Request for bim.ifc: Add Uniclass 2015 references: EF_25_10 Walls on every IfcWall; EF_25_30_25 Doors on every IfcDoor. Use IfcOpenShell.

First a look at what the model holds.

```python
import ifcopenshell

model = ifcopenshell.open("bim.ifc")
print(model.schema)
print("classifications:", [c.Name for c in model.by_type("IfcClassification")])
for ifc_class in ("IfcDoor", "IfcRoof", "IfcStair", "IfcWall", "IfcWindow"):
    print(ifc_class, len(model.by_type(ifc_class)))
```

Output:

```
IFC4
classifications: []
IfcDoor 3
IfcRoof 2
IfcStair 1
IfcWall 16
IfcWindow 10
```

```python
import ifcopenshell
import ifcopenshell.api.classification

model = ifcopenshell.open("bim.ifc")

system = ifcopenshell.api.classification.add_classification(model, classification="Uniclass 2015")

codes = {
    "IfcWall": ("EF_25_10", "Walls"),
    "IfcDoor": ("EF_25_30_25", "Doors"),
}
for ifc_class, (code, name) in codes.items():
    products = model.by_type(ifc_class)
    ifcopenshell.api.classification.add_reference(
        model, products=products, classification=system, identification=code, name=name
    )
    print(code, len(products))

model.write("bim-out.ifc")
```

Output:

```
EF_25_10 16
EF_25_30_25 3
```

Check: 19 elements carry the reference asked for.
